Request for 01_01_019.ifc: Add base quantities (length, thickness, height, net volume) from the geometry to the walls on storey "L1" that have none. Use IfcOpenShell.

First a look at what the model holds.

```python
import ifcopenshell
import ifcopenshell.util.element
import ifcopenshell.util.unit

model = ifcopenshell.open("01_01_019.ifc")
print(model.schema)
for unit_type in ("LENGTHUNIT", "AREAUNIT", "VOLUMEUNIT"):
    print(unit_type, ifcopenshell.util.unit.calculate_unit_scale(model, unit_type))
storey = next(s for s in model.by_type("IfcBuildingStorey") if s.Name == "L1")
walls = [e for e in ifcopenshell.util.element.get_decomposition(storey) if e.is_a("IfcWall")]
for e in sorted(walls, key=lambda e: e.id()):
    print(e.id(), e.is_a(), e.Name, list(ifcopenshell.util.element.get_psets(e, qtos_only=True)), sep=" | ")
```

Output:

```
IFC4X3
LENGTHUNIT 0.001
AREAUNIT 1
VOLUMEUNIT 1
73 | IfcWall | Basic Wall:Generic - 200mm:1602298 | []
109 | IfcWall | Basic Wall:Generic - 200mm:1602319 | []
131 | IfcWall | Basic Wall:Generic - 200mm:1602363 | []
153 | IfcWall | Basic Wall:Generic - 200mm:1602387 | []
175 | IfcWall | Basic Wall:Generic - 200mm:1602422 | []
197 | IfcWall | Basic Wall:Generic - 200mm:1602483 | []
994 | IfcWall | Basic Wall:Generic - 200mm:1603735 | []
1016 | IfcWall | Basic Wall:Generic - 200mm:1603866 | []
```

```python
import ifcopenshell
import ifcopenshell.api.pset
import ifcopenshell.geom
import ifcopenshell.util.element
import ifcopenshell.util.shape
import ifcopenshell.util.unit

model = ifcopenshell.open("01_01_019.ifc")
unit_scale = ifcopenshell.util.unit.calculate_unit_scale(model)
volume_scale = ifcopenshell.util.unit.calculate_unit_scale(model, "VOLUMEUNIT")
settings = ifcopenshell.geom.settings()

storey = next(s for s in model.by_type("IfcBuildingStorey") if s.Name == "L1")
walls = [e for e in ifcopenshell.util.element.get_decomposition(storey) if e.is_a("IfcWall")]

for e in sorted(walls, key=lambda e: e.id()):
    if ifcopenshell.util.element.get_psets(e, qtos_only=True, should_inherit=False):
        continue
    # Geometry comes back in metres, in the element's own axes.
    shape = ifcopenshell.geom.create_shape(settings, e)
    values = {
        "Length": ifcopenshell.util.shape.get_x(shape.geometry) / unit_scale,
        "Width": ifcopenshell.util.shape.get_y(shape.geometry) / unit_scale,
        "Height": ifcopenshell.util.shape.get_z(shape.geometry) / unit_scale,
        "NetVolume": ifcopenshell.util.shape.get_volume(shape.geometry) / volume_scale,
    }
    qto = ifcopenshell.api.pset.add_qto(model, product=e, name="Qto_WallBaseQuantities")
    ifcopenshell.api.pset.edit_qto(model, qto=qto, properties=values)
    print(e.id(), {k: round(v, 3) for k, v in values.items()})

model.write("01_01_019_rev.ifc")
```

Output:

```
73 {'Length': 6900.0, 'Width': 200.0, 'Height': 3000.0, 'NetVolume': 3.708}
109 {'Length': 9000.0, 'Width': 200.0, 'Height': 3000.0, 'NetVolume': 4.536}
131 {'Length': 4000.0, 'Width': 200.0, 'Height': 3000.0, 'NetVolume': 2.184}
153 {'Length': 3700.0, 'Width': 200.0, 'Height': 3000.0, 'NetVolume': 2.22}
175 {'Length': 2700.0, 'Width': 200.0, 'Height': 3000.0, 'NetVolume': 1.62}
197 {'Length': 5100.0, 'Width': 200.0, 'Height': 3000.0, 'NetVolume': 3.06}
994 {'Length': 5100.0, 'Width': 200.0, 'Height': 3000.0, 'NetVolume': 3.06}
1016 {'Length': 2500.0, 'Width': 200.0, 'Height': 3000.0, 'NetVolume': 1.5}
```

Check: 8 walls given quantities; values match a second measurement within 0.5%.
